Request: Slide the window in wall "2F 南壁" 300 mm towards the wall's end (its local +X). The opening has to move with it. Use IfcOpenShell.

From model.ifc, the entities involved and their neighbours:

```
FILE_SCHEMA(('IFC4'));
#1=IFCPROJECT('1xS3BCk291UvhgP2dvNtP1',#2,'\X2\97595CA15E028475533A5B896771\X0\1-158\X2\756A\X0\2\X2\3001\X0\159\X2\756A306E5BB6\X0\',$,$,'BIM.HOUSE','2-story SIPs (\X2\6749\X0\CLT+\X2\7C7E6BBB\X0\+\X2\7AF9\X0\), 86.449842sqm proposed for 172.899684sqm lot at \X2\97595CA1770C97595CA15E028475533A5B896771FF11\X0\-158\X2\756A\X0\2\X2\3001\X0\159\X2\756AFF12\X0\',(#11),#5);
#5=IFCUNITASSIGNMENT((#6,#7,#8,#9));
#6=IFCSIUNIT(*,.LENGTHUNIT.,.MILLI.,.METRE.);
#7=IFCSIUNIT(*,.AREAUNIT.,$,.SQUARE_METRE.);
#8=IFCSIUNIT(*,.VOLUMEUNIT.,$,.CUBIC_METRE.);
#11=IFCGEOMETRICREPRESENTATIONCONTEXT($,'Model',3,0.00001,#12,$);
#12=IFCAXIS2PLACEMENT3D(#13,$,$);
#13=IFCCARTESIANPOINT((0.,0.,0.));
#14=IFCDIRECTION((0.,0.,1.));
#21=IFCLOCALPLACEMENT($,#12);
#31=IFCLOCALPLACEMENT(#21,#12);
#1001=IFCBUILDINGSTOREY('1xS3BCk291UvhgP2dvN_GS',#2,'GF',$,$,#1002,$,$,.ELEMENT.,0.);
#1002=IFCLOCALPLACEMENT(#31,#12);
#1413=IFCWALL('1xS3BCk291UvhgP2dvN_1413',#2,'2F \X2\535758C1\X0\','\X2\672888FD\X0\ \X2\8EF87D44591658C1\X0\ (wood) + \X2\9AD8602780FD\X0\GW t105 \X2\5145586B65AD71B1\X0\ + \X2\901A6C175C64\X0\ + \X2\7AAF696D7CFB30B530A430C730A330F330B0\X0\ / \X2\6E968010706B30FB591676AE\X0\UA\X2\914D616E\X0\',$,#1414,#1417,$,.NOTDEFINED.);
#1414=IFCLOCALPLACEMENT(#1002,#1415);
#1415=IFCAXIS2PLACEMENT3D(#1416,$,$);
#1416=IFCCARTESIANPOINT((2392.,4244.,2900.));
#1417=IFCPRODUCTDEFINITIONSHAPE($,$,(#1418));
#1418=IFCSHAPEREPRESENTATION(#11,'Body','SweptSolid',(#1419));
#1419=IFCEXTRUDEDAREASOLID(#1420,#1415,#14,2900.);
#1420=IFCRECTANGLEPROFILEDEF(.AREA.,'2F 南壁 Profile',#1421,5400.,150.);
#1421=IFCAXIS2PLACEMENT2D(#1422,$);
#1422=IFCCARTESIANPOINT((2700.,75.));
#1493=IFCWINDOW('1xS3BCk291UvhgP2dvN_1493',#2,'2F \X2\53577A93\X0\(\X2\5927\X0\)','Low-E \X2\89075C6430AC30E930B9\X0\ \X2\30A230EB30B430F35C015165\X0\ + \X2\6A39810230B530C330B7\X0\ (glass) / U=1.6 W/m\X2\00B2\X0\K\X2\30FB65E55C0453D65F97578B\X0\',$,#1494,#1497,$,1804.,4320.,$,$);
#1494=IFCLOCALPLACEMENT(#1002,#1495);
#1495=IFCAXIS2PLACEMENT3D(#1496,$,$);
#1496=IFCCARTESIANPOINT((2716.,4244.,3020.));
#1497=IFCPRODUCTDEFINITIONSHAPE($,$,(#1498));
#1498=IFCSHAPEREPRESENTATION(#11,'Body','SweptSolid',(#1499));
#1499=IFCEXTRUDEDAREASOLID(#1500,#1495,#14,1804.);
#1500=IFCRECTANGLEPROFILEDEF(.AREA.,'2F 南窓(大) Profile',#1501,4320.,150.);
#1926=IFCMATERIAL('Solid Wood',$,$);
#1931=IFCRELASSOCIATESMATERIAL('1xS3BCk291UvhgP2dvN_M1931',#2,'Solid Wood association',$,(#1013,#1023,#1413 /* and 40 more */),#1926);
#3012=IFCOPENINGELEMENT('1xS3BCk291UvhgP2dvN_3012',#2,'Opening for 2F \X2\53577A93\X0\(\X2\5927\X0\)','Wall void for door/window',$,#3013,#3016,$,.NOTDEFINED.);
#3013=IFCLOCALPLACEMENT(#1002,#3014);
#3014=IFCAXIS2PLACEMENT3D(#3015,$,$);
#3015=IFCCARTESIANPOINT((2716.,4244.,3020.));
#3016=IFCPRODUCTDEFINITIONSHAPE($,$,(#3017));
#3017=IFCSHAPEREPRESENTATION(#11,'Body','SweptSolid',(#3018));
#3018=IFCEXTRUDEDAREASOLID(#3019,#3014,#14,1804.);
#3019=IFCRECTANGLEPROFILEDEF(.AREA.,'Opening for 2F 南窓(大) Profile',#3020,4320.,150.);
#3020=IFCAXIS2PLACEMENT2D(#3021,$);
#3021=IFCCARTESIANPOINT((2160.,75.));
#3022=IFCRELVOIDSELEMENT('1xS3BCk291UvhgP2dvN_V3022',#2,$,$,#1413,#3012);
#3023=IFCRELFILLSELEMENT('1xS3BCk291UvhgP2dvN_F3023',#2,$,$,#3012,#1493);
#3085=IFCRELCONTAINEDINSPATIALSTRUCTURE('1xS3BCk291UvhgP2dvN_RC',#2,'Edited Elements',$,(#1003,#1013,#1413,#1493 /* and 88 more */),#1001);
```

```python
import ifcopenshell
import ifcopenshell.api.geometry
import ifcopenshell.util.placement

model = ifcopenshell.open("model.ifc")

window = model.by_guid("1xS3BCk291UvhgP2dvN_1493")
opening = window.FillsVoids[0].RelatingOpeningElement
wall = opening.VoidsElements[0].RelatingBuildingElement

wall_matrix = ifcopenshell.util.placement.get_local_placement(wall.ObjectPlacement)
shift = wall_matrix[:3, 0] * 300.0
before = ifcopenshell.util.placement.get_local_placement(window.ObjectPlacement)[:3, 3].copy()

# The window is not placed relative to its opening, so move both.
for product in (opening, window):
    matrix = ifcopenshell.util.placement.get_local_placement(product.ObjectPlacement)
    matrix[:3, 3] += shift
    ifcopenshell.api.geometry.edit_object_placement(model, product=product, matrix=matrix, is_si=False)

after = ifcopenshell.util.placement.get_local_placement(window.ObjectPlacement)[:3, 3]
print("window moved by", (after - before).round(3) + 0.0)

model.write("model_updated.ifc")
```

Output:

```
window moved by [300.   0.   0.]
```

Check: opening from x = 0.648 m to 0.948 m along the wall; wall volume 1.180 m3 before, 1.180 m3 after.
